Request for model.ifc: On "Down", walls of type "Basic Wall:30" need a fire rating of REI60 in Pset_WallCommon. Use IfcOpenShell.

First a look at what the model holds.

```python
import ifcopenshell
import ifcopenshell.util.element

model = ifcopenshell.open("model.ifc")
print(model.schema)
storey = next(s for s in model.by_type("IfcBuildingStorey") if s.Name == "Down")
walls = [e for e in ifcopenshell.util.element.get_decomposition(storey) if e.is_a("IfcWall")]
seen = {}
for e in walls:
    element_type = ifcopenshell.util.element.get_type(e)
    key = (element_type.Name if element_type != e and element_type else None, ifcopenshell.util.element.get_pset(e, "Pset_WallCommon", "FireRating"))
    seen[key] = seen.get(key, 0) + 1
for (name, value), count in sorted(seen.items(), key=str):
    print(count, "x", name, "|", value)
```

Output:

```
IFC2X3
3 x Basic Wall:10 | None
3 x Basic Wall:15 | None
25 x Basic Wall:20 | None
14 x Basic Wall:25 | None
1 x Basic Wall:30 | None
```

```python
import ifcopenshell
import ifcopenshell.api.pset
import ifcopenshell.util.element

model = ifcopenshell.open("model.ifc")

storey = next(s for s in model.by_type("IfcBuildingStorey") if s.Name == "Down")
walls = [e for e in ifcopenshell.util.element.get_decomposition(storey) if e.is_a("IfcWall")]

count = 0
for e in walls:
    element_type = ifcopenshell.util.element.get_type(e)
    if element_type in (None, e) or element_type.Name != "Basic Wall:30":
        continue
    # add_pset returns the element's existing set when there is one.
    pset = ifcopenshell.api.pset.add_pset(model, product=e, name="Pset_WallCommon")
    ifcopenshell.api.pset.edit_pset(model, pset=pset, properties={"FireRating": "REI60"})
    count += 1

print(count, "walls updated")

model.write("model_updated.ifc")
```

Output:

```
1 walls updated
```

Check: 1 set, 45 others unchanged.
